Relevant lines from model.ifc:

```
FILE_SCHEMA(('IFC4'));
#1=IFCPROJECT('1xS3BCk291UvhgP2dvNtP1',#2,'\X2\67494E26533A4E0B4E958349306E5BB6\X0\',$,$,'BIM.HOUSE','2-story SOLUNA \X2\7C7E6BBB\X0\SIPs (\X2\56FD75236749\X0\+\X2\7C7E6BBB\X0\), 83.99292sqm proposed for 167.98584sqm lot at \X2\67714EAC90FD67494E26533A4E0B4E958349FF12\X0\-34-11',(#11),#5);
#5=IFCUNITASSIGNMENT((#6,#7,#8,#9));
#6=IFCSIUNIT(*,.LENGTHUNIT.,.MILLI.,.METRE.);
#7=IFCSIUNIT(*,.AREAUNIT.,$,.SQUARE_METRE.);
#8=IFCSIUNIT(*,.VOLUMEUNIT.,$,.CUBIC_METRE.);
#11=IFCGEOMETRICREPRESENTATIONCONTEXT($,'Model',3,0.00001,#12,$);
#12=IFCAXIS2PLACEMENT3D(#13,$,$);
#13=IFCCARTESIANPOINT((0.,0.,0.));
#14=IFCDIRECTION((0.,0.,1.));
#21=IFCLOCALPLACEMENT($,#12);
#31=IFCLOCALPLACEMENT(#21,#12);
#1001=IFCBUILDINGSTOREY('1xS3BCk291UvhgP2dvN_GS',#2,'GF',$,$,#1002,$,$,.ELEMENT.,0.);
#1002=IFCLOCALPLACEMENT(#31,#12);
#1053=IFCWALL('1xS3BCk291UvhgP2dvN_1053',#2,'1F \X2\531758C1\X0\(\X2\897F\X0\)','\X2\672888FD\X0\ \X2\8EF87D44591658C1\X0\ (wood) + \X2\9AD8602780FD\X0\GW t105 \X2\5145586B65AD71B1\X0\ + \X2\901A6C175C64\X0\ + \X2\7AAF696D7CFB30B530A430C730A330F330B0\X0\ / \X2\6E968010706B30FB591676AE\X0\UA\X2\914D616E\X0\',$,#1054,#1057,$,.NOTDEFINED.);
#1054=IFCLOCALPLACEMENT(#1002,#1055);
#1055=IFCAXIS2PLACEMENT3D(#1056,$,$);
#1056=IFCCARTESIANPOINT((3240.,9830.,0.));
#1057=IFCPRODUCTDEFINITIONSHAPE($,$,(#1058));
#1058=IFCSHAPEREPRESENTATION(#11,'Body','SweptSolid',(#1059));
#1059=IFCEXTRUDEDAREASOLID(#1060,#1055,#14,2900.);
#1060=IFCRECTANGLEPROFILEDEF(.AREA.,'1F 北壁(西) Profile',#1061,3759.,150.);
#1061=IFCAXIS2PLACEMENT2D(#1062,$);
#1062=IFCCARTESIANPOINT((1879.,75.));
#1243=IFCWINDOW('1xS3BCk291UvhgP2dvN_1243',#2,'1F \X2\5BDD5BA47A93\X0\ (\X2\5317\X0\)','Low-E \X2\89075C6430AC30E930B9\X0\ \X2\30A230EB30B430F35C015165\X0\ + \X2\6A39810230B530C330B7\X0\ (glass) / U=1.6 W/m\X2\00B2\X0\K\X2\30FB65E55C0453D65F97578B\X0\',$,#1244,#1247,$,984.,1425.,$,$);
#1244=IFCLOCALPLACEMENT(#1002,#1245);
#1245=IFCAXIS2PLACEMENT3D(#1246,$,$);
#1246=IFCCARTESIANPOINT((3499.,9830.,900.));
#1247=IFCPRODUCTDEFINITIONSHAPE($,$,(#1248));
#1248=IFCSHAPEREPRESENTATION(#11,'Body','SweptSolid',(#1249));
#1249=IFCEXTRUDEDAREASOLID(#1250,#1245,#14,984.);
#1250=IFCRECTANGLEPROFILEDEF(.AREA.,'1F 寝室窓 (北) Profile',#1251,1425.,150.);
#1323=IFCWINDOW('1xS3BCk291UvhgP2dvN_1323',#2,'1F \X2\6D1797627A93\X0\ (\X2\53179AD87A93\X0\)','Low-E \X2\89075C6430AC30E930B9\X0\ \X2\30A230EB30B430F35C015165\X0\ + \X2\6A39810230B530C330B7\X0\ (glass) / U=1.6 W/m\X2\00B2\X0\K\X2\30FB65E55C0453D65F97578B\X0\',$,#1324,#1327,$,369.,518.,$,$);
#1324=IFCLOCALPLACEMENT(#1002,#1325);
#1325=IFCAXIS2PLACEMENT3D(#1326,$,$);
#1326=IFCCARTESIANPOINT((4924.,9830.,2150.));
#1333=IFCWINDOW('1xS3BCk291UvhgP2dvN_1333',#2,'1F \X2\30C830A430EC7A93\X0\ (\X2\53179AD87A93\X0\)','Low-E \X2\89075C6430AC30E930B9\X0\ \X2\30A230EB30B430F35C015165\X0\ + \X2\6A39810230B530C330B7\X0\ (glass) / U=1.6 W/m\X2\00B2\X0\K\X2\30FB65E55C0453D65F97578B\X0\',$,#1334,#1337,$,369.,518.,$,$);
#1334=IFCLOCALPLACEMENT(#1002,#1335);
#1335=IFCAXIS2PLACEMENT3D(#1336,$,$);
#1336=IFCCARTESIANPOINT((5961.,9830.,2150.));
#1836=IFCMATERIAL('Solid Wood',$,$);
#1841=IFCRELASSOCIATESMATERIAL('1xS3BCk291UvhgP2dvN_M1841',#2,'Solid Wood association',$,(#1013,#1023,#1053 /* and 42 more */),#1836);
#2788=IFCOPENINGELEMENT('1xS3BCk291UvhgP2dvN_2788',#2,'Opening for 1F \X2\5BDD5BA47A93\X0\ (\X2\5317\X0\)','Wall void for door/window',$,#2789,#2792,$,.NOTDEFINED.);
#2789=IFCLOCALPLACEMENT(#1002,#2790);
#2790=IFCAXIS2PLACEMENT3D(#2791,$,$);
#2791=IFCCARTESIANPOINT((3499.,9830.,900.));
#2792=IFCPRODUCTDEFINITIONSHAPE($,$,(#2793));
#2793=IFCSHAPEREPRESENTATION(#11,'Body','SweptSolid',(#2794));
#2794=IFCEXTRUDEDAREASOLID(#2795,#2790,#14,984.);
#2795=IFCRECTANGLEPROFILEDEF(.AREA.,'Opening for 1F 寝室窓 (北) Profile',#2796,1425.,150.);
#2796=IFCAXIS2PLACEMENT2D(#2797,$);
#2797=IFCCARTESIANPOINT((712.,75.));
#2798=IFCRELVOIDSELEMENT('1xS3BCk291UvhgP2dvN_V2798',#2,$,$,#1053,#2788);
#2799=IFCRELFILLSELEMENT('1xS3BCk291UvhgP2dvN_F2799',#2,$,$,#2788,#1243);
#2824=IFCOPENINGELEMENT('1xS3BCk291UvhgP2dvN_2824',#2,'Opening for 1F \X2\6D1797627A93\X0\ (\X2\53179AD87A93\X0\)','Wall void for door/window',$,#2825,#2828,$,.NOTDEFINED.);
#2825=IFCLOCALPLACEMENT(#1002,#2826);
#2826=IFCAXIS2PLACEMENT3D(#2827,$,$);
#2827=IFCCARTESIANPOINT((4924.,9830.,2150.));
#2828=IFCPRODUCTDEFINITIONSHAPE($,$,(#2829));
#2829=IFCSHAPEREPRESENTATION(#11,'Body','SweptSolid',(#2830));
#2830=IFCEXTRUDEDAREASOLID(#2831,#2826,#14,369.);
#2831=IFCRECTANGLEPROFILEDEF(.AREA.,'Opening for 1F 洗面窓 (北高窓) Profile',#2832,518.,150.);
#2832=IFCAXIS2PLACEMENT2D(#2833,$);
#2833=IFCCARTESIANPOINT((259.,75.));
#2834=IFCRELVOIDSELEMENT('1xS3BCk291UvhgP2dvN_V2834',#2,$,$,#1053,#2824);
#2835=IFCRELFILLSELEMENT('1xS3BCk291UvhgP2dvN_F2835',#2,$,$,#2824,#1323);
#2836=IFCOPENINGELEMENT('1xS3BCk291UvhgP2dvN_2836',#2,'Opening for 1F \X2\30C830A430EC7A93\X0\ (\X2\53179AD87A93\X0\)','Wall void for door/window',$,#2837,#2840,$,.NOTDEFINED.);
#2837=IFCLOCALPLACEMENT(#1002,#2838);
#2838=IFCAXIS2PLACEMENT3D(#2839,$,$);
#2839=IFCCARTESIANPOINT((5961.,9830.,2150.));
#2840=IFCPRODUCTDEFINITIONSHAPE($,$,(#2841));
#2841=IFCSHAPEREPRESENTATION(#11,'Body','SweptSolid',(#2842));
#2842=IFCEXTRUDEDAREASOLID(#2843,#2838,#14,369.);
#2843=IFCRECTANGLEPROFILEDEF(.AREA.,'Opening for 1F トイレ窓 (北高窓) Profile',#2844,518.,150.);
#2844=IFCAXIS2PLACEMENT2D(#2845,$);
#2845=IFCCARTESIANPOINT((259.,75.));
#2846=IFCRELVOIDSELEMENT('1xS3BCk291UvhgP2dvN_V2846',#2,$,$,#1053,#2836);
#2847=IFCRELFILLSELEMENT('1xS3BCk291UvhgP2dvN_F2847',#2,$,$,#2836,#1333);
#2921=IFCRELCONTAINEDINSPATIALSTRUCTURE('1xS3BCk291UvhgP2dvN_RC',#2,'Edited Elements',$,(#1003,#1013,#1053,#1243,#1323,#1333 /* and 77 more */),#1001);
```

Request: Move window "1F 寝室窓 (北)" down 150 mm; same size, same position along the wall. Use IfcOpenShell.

```python
import numpy as np
import ifcopenshell
import ifcopenshell.api.geometry
import ifcopenshell.util.placement
import ifcopenshell.util.unit

model = ifcopenshell.open("model.ifc")
unit_scale = ifcopenshell.util.unit.calculate_unit_scale(model)

window = model.by_id(1243)
opening = window.FillsVoids[0].RelatingOpeningElement
dz = -0.15 / unit_scale

shift = np.array([0.0, 0.0, dz])
# The window is not placed relative to its opening, so move both.
for product in (opening, window):
    matrix = ifcopenshell.util.placement.get_local_placement(product.ObjectPlacement)
    matrix[:3, 3] += shift
    ifcopenshell.api.geometry.edit_object_placement(model, product=product, matrix=matrix, is_si=False)

print(f"moved by {dz * unit_scale:+.3f} m")

model.write("model_updated.ifc")
```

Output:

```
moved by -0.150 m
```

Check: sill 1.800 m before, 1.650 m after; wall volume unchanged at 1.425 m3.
